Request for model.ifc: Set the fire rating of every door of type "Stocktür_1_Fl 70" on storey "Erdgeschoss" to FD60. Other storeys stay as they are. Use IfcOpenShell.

First a look at what the model holds.

```python
import ifcopenshell
import ifcopenshell.util.element

model = ifcopenshell.open("model.ifc")
print(model.schema)
storey = next(s for s in model.by_type("IfcBuildingStorey") if s.Name == "Erdgeschoss")
doors = [e for e in ifcopenshell.util.element.get_decomposition(storey) if e.is_a("IfcDoor")]
seen = {}
for e in doors:
    element_type = ifcopenshell.util.element.get_type(e)
    key = (element_type.Name if element_type != e and element_type else None, ifcopenshell.util.element.get_pset(e, "Pset_DoorCommon", "FireRating"))
    seen[key] = seen.get(key, 0) + 1
for (name, value), count in sorted(seen.items(), key=str):
    print(count, "x", name, "|", value)
```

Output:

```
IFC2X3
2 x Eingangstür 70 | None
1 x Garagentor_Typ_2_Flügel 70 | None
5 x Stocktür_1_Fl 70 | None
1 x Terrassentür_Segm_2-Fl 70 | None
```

```python
import ifcopenshell
import ifcopenshell.api.pset
import ifcopenshell.util.element

model = ifcopenshell.open("model.ifc")

storey = next(s for s in model.by_type("IfcBuildingStorey") if s.Name == "Erdgeschoss")
doors = [e for e in ifcopenshell.util.element.get_decomposition(storey) if e.is_a("IfcDoor")]

count = 0
for e in doors:
    element_type = ifcopenshell.util.element.get_type(e)
    if element_type in (None, e) or element_type.Name != "Stocktür_1_Fl 70":
        continue
    # add_pset returns the element's existing set when there is one.
    pset = ifcopenshell.api.pset.add_pset(model, product=e, name="Pset_DoorCommon")
    ifcopenshell.api.pset.edit_pset(model, pset=pset, properties={"FireRating": "FD60"})
    count += 1

print(count, "doors updated")

model.write("model_edited.ifc")
```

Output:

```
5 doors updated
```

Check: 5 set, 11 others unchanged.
